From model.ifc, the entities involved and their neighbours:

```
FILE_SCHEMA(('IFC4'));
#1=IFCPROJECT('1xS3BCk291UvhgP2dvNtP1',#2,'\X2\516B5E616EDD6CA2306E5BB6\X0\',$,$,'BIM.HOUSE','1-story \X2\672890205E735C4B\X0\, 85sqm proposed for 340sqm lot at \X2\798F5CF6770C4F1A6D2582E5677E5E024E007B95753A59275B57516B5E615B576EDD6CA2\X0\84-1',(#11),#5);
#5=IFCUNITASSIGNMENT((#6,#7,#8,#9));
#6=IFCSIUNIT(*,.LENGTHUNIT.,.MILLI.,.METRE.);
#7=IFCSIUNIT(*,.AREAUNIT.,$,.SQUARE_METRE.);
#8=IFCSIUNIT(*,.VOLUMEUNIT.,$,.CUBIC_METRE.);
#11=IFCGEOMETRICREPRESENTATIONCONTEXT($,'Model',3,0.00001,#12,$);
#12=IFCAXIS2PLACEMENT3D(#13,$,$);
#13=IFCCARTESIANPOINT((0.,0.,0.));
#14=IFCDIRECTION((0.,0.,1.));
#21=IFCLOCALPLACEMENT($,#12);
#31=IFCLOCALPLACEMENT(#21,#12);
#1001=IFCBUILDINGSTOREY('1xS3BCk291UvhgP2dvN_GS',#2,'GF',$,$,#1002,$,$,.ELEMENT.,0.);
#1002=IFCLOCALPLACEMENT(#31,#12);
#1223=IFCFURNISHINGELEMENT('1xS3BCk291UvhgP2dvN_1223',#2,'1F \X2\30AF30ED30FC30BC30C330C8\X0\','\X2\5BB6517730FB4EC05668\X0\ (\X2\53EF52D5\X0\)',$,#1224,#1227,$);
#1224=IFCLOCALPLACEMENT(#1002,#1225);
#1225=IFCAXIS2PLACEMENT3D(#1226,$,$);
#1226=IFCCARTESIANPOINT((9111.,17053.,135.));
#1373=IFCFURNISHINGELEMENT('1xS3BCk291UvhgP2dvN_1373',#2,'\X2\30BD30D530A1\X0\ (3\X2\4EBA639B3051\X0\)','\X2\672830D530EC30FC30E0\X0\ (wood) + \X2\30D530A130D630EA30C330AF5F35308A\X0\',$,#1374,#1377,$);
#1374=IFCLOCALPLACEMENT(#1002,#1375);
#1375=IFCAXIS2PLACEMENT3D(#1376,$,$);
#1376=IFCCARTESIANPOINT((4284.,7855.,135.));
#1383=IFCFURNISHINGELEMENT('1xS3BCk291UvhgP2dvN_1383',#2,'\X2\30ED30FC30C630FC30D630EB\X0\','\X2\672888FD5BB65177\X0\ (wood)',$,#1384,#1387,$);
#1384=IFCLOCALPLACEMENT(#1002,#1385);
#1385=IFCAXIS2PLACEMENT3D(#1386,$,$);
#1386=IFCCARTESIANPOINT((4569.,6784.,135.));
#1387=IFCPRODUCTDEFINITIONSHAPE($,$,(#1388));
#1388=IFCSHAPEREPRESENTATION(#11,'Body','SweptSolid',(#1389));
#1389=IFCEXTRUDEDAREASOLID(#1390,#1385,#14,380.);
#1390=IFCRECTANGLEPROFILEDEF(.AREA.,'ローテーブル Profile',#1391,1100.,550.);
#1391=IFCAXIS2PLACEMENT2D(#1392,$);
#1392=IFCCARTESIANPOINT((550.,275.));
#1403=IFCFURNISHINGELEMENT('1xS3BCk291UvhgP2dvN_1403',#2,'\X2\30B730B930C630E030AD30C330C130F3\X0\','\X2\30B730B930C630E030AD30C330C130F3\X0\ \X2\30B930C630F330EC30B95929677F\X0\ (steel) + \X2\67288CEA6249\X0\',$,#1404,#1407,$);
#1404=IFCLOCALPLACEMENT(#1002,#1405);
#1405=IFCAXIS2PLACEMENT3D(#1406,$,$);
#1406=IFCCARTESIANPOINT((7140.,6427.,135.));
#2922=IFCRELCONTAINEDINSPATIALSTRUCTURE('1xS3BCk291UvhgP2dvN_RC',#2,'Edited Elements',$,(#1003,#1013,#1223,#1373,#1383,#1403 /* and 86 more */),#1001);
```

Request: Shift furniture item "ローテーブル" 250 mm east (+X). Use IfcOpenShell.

```python
import ifcopenshell
import ifcopenshell.api.geometry
import ifcopenshell.util.placement
import ifcopenshell.util.unit

model = ifcopenshell.open("model.ifc")
unit_scale = ifcopenshell.util.unit.calculate_unit_scale(model)

item = model.by_guid("1xS3BCk291UvhgP2dvN_1383")
matrix = ifcopenshell.util.placement.get_local_placement(item.ObjectPlacement)
matrix[0, 3] += 0.25 / unit_scale
ifcopenshell.api.geometry.edit_object_placement(model, product=item, matrix=matrix, is_si=False)

print(ifcopenshell.util.placement.get_local_placement(item.ObjectPlacement).round(3) + 0.0)

model.write("model_updated.ifc")
```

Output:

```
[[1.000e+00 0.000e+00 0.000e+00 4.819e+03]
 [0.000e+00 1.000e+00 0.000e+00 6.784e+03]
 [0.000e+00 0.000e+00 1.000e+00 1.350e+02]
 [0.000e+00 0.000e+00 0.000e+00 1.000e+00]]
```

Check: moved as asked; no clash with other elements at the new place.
